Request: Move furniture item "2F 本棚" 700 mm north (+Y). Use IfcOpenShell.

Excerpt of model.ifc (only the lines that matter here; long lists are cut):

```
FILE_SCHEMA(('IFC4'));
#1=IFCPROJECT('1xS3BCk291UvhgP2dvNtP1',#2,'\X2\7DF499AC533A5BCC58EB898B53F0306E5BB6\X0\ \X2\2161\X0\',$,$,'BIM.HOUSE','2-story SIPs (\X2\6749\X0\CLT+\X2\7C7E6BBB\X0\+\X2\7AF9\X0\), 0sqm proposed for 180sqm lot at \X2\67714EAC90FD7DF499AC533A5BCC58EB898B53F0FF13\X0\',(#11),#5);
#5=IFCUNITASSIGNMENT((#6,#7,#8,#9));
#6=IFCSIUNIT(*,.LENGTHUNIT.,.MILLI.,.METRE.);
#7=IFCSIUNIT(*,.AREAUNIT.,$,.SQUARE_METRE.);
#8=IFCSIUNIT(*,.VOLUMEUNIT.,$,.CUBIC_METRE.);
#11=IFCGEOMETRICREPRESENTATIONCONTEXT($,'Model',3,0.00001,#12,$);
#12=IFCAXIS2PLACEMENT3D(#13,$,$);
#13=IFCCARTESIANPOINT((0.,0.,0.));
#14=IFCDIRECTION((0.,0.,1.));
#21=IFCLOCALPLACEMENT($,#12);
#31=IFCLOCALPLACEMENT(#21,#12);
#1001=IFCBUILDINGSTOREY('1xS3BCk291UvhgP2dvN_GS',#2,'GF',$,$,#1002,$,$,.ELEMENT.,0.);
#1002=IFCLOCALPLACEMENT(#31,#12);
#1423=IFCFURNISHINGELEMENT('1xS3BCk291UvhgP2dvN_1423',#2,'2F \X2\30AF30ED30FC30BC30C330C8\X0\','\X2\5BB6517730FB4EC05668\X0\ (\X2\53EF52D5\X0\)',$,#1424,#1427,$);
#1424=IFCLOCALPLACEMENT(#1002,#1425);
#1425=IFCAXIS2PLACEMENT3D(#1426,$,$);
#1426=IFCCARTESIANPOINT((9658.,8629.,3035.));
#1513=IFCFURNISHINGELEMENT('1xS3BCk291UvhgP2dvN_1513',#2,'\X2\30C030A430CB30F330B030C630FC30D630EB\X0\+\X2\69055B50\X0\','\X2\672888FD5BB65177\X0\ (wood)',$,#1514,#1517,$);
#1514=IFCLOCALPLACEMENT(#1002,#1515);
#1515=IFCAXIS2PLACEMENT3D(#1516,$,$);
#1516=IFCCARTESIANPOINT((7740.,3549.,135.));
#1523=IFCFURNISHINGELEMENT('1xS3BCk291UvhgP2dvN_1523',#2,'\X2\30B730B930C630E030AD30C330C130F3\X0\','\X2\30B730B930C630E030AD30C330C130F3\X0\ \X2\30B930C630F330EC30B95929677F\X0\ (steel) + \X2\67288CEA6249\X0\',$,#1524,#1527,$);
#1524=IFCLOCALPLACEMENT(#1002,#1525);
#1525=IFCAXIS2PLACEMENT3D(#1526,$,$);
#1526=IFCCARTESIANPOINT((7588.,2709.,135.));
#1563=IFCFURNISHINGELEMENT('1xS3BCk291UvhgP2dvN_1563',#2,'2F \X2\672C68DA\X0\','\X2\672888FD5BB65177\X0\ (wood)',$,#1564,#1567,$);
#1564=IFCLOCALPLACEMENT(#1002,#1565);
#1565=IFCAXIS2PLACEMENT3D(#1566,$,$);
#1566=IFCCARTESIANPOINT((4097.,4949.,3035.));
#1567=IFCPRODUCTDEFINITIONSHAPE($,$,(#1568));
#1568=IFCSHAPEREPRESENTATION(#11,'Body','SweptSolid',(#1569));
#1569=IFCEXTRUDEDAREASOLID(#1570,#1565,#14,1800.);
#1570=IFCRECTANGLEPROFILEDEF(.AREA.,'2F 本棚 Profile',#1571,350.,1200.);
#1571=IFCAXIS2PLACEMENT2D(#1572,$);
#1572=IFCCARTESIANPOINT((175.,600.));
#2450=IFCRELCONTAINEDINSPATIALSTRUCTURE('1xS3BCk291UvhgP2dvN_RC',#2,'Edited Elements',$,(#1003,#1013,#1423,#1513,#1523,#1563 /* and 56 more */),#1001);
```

```python
import ifcopenshell
import ifcopenshell.api.geometry
import ifcopenshell.util.placement

model = ifcopenshell.open("model.ifc")

item = model.by_id(1563)
matrix = ifcopenshell.util.placement.get_local_placement(item.ObjectPlacement)
matrix[1, 3] += 700.0
ifcopenshell.api.geometry.edit_object_placement(model, product=item, matrix=matrix, is_si=False)

print(ifcopenshell.util.placement.get_local_placement(item.ObjectPlacement).round(3) + 0.0)

model.write("model_rev.ifc")
```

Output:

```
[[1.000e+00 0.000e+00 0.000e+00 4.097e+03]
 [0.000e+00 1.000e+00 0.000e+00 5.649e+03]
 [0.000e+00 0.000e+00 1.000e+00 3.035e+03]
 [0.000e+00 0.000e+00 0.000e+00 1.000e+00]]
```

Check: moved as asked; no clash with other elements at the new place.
